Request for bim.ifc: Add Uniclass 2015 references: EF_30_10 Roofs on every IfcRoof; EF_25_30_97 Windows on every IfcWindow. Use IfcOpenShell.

First a look at what the model holds.

```python
import ifcopenshell

model = ifcopenshell.open("bim.ifc")
print(model.schema)
print("classifications:", [c.Name for c in model.by_type("IfcClassification")])
for ifc_class in ("IfcDoor", "IfcRoof", "IfcStair", "IfcWall", "IfcWindow"):
    print(ifc_class, len(model.by_type(ifc_class)))
```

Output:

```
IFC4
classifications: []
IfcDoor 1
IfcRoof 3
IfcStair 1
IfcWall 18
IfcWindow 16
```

```python
import ifcopenshell
import ifcopenshell.api.classification

model = ifcopenshell.open("bim.ifc")

system = ifcopenshell.api.classification.add_classification(model, classification="Uniclass 2015")

codes = {
    "IfcRoof": ("EF_30_10", "Roofs"),
    "IfcWindow": ("EF_25_30_97", "Windows"),
}
for ifc_class, (code, name) in codes.items():
    products = model.by_type(ifc_class)
    ifcopenshell.api.classification.add_reference(
        model, products=products, classification=system, identification=code, name=name
    )
    print(code, len(products))

model.write("bim_edited.ifc")
```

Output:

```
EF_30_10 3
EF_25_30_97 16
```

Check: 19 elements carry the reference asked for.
